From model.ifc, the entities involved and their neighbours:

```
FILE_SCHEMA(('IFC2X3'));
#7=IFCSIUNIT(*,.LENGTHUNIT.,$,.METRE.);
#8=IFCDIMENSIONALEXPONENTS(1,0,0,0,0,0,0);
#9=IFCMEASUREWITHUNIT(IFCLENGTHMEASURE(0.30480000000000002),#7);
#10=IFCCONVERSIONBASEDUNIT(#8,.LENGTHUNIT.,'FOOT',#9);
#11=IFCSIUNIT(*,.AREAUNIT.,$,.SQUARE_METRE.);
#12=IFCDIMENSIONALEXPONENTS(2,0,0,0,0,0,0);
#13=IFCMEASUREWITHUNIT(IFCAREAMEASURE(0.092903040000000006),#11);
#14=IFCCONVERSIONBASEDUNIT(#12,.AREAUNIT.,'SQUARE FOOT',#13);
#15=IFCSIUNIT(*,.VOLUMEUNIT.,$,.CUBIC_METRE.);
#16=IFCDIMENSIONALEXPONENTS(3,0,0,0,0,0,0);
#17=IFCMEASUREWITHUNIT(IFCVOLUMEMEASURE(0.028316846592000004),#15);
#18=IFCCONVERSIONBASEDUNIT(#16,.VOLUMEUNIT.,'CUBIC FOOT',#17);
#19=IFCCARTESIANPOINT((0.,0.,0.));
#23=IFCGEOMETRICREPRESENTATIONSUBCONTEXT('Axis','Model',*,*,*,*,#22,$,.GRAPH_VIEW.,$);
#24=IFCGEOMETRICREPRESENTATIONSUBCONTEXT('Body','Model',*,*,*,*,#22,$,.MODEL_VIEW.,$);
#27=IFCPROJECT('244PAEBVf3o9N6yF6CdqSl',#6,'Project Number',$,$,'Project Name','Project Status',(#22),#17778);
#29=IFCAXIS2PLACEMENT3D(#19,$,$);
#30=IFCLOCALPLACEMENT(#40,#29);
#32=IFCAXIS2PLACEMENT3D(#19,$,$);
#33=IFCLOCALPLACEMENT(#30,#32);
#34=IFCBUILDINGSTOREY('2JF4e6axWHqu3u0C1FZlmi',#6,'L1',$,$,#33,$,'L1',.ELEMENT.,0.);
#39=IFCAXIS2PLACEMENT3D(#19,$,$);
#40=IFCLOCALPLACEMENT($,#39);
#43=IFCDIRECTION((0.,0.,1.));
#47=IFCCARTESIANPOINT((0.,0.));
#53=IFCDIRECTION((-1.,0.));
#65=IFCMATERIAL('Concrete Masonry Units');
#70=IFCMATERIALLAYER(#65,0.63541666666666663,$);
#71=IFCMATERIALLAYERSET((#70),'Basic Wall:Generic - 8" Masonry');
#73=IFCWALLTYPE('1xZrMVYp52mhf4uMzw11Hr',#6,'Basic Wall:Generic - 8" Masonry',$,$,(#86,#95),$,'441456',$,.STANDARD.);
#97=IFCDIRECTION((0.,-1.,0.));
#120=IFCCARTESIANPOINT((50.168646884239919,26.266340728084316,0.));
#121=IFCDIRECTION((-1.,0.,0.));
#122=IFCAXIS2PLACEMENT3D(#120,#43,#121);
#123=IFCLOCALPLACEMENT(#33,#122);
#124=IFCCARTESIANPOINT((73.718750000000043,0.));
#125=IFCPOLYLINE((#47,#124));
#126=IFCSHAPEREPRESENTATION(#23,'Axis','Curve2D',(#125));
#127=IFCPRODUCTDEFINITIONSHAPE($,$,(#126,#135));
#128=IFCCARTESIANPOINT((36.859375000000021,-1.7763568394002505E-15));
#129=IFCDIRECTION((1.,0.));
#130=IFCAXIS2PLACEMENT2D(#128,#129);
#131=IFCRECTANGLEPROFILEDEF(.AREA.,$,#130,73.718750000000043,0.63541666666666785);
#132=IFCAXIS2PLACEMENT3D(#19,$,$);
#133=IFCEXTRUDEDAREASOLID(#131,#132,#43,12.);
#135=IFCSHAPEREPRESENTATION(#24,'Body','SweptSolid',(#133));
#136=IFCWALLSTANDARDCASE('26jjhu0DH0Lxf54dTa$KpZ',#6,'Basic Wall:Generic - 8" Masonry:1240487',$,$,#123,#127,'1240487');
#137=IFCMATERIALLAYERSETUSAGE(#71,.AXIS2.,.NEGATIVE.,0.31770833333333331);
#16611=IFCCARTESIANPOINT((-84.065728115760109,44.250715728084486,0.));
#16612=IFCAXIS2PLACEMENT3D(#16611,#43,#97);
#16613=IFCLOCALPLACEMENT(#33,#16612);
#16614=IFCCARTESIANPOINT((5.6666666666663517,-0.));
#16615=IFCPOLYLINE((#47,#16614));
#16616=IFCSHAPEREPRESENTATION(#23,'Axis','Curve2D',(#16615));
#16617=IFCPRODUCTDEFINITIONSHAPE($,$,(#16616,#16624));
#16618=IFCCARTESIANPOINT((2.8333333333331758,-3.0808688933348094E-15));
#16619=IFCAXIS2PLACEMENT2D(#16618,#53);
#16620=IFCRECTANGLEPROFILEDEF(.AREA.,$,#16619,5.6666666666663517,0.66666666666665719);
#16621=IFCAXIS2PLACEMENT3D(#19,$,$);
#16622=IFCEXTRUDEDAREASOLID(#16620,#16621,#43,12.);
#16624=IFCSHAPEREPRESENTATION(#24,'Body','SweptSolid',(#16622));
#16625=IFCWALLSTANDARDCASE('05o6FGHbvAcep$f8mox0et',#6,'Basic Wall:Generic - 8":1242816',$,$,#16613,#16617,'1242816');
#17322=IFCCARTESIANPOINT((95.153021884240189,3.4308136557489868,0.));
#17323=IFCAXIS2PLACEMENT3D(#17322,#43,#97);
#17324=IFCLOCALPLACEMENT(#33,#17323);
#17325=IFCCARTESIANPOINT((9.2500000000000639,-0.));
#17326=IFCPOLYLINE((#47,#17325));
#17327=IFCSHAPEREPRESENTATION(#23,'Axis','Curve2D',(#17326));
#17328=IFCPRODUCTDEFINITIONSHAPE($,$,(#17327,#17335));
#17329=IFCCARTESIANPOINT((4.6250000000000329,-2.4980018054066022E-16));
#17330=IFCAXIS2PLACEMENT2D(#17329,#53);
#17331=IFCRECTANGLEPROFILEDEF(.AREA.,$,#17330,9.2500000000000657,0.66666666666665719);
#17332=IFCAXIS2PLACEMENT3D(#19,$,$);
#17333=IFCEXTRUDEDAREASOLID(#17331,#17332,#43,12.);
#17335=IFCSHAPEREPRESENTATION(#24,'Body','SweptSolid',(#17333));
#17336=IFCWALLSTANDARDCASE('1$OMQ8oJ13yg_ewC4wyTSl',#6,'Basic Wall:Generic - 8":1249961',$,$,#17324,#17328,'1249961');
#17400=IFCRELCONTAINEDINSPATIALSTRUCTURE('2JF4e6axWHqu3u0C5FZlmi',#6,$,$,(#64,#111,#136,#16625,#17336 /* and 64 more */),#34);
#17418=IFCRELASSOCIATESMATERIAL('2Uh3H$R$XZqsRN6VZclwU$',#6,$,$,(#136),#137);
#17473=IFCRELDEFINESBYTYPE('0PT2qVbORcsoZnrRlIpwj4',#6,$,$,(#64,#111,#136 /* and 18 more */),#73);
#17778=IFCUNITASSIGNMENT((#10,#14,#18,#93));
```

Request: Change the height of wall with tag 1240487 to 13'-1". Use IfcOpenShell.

```python
import ifcopenshell
import ifcopenshell.geom
import ifcopenshell.util.representation
import ifcopenshell.util.shape
import ifcopenshell.util.unit

model = ifcopenshell.open("model.ifc")
unit_scale = ifcopenshell.util.unit.calculate_unit_scale(model)
settings = ifcopenshell.geom.settings()


def volume(element):
    """Net volume in cubic metres, openings subtracted."""
    shape = ifcopenshell.geom.create_shape(settings, element)
    return ifcopenshell.util.shape.get_volume(shape.geometry)


wall = model.by_guid("26jjhu0DH0Lxf54dTa$KpZ")
before = volume(wall)

body = ifcopenshell.util.representation.get_representation(wall, "Model", "Body")
solid = body.Items[0]
old_height = solid.Depth
solid.Depth = 157 * 0.0254 / unit_scale
after = volume(wall)

print(f"height {old_height:g} -> {solid.Depth:g}, volume {before:.3f} -> {after:.3f} m3")

model.write("model_edited.ifc")
```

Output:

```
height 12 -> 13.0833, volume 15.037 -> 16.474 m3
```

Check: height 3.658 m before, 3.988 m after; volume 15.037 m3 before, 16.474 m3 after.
